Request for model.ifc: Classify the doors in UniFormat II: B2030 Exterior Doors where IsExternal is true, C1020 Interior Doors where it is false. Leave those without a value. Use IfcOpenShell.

First a look at what the model holds.

```python
import ifcopenshell
import ifcopenshell.util.element

model = ifcopenshell.open("model.ifc")
print(model.schema)
print("classifications:", [c.Name for c in model.by_type("IfcClassification")])
values = [ifcopenshell.util.element.get_pset(e, "Pset_DoorCommon", "IsExternal") for e in model.by_type("IfcDoor")]
for value in (True, False, None):
    print("IsExternal", value, values.count(value))
```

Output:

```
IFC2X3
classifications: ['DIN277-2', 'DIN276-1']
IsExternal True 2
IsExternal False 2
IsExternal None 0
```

```python
import ifcopenshell
import ifcopenshell.api.classification
import ifcopenshell.util.element

model = ifcopenshell.open("model.ifc")

# IFC2X3 requires Source and Edition and has no link from the project to the system.
system = model.create_entity("IfcClassification", Source="ASTM", Edition="E1557", Name="UniFormat II")

doors = model.by_type("IfcDoor")
external = {e: ifcopenshell.util.element.get_pset(e, "Pset_DoorCommon", "IsExternal") for e in doors}
for flag, code, name in ((True, "B2030", "Exterior Doors"), (False, "C1020", "Interior Doors")):
    products = [e for e in doors if external[e] is flag]
    ifcopenshell.api.classification.add_reference(
        model, products=products, classification=system, identification=code, name=name
    )
    print(code, len(products))

model.write("model_v2.ifc")
```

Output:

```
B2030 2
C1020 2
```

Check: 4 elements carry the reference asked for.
